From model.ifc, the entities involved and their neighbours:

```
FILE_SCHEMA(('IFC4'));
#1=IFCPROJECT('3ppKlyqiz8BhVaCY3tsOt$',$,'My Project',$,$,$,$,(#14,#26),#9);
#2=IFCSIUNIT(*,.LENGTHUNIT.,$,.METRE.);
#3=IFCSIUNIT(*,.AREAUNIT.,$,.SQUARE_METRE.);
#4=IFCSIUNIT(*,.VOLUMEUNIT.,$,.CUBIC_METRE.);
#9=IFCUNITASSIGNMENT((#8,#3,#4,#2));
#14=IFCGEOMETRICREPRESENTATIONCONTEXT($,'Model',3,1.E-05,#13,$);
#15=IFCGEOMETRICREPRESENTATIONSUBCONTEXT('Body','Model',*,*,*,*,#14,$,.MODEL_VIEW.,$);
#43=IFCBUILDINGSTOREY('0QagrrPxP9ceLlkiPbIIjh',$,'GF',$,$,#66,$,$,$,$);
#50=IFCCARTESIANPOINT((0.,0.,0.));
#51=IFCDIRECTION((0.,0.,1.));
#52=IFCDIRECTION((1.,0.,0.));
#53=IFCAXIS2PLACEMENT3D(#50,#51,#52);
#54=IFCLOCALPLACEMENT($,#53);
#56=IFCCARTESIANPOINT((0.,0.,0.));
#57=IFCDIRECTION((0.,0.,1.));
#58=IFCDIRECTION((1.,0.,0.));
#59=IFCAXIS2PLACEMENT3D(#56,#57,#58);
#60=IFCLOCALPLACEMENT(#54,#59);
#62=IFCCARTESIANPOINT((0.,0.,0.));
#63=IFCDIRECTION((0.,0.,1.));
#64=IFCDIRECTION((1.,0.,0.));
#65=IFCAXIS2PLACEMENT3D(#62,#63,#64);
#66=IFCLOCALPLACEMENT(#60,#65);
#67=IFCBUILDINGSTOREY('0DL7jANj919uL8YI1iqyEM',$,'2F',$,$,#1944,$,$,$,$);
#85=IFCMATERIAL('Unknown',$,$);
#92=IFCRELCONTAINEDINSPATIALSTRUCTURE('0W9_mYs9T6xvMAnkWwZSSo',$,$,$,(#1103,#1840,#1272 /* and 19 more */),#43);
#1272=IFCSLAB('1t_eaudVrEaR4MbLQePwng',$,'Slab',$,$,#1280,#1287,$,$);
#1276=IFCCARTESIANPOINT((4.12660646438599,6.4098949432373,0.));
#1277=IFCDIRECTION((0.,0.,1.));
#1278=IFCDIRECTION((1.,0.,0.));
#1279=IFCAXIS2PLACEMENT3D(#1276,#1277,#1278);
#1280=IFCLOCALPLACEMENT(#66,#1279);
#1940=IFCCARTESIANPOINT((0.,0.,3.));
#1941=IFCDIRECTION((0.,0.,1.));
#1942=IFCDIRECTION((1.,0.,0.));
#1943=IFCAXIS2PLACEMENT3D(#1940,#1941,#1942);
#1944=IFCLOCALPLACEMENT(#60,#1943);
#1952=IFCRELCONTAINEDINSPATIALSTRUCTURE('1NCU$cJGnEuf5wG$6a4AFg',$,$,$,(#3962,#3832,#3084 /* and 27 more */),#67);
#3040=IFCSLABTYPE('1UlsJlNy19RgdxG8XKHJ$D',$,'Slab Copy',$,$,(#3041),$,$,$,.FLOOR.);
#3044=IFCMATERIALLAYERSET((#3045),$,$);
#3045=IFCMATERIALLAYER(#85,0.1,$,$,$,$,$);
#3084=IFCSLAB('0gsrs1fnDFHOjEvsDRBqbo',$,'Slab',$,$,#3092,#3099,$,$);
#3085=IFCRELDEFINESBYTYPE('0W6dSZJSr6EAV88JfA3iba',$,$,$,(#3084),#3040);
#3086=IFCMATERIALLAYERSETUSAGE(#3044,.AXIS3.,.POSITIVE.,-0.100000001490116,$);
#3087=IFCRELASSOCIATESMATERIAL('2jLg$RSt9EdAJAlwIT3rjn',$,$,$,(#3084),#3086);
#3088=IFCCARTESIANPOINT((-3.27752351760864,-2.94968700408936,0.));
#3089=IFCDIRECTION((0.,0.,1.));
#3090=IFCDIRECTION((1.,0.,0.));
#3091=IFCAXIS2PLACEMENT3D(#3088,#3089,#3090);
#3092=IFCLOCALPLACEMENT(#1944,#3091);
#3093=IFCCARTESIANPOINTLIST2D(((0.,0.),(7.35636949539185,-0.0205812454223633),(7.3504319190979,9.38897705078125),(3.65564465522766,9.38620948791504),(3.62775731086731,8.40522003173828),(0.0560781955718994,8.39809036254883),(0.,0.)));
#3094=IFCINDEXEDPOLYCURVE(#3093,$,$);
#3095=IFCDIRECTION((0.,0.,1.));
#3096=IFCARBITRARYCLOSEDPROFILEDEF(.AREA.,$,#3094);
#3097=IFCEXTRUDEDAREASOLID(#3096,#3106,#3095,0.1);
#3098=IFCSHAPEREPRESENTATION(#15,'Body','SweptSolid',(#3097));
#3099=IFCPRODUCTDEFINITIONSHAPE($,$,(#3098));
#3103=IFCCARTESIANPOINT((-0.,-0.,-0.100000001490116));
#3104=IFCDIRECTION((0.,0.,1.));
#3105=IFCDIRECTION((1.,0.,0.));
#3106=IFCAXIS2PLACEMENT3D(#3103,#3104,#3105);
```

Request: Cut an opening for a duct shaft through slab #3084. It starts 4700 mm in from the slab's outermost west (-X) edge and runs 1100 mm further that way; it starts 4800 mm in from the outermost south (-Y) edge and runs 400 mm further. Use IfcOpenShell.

```python
import numpy as np
import ifcopenshell
import ifcopenshell.api.feature
import ifcopenshell.api.geometry
import ifcopenshell.api.root
import ifcopenshell.geom
import ifcopenshell.util.placement
import ifcopenshell.util.representation
import ifcopenshell.util.shape
import ifcopenshell.util.unit

model = ifcopenshell.open("model.ifc")
unit_scale = ifcopenshell.util.unit.calculate_unit_scale(model)
settings = ifcopenshell.geom.settings()


def volume(element):
    """Net volume in cubic metres, openings subtracted."""
    shape = ifcopenshell.geom.create_shape(settings, element)
    return ifcopenshell.util.shape.get_volume(shape.geometry)


slab = model.by_guid("0gsrs1fnDFHOjEvsDRBqbo")
before = volume(slab)

# Extent in the slab's own axes, in metres. The edges named are its -X and -Y sides.
slab_shape = ifcopenshell.geom.create_shape(settings, slab)
vertices = ifcopenshell.util.shape.get_vertices(slab_shape.geometry)
x_min, y_min, bottom = vertices.min(axis=0)
top = vertices[:, 2].max()

opening = ifcopenshell.api.root.create_entity(model, ifc_class="IfcOpeningElement", name="Duct shaft opening", predefined_type="OPENING")
context = ifcopenshell.util.representation.get_context(model, "Model", "Body", "MODEL_VIEW")
width, depth = 1.1, 0.4
outline = [(0.0, 0.0), (width, 0.0), (width, depth), (0.0, depth), (0.0, 0.0)]
# Overshoot both faces by 50 mm so the cut is clean.
shape = ifcopenshell.api.geometry.add_slab_representation(
    model, context=context, depth=top - bottom + 0.1, polyline=outline
)
ifcopenshell.api.geometry.assign_representation(model, product=opening, representation=shape)

matrix = ifcopenshell.util.placement.get_local_placement(slab.ObjectPlacement)
matrix[:, 3] = matrix @ np.append(np.array([x_min + 4.7, y_min + 4.8, bottom - 0.05]) / unit_scale, 1.0)
ifcopenshell.api.geometry.edit_object_placement(model, product=opening, matrix=matrix, is_si=False)
ifcopenshell.api.feature.add_feature(model, feature=opening, element=slab)

after = volume(slab)

print(f"slab volume {before:.3f} -> {after:.3f} m3")

model.write("model-out.ifc")
```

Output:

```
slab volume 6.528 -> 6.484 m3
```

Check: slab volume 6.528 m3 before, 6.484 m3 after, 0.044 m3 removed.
